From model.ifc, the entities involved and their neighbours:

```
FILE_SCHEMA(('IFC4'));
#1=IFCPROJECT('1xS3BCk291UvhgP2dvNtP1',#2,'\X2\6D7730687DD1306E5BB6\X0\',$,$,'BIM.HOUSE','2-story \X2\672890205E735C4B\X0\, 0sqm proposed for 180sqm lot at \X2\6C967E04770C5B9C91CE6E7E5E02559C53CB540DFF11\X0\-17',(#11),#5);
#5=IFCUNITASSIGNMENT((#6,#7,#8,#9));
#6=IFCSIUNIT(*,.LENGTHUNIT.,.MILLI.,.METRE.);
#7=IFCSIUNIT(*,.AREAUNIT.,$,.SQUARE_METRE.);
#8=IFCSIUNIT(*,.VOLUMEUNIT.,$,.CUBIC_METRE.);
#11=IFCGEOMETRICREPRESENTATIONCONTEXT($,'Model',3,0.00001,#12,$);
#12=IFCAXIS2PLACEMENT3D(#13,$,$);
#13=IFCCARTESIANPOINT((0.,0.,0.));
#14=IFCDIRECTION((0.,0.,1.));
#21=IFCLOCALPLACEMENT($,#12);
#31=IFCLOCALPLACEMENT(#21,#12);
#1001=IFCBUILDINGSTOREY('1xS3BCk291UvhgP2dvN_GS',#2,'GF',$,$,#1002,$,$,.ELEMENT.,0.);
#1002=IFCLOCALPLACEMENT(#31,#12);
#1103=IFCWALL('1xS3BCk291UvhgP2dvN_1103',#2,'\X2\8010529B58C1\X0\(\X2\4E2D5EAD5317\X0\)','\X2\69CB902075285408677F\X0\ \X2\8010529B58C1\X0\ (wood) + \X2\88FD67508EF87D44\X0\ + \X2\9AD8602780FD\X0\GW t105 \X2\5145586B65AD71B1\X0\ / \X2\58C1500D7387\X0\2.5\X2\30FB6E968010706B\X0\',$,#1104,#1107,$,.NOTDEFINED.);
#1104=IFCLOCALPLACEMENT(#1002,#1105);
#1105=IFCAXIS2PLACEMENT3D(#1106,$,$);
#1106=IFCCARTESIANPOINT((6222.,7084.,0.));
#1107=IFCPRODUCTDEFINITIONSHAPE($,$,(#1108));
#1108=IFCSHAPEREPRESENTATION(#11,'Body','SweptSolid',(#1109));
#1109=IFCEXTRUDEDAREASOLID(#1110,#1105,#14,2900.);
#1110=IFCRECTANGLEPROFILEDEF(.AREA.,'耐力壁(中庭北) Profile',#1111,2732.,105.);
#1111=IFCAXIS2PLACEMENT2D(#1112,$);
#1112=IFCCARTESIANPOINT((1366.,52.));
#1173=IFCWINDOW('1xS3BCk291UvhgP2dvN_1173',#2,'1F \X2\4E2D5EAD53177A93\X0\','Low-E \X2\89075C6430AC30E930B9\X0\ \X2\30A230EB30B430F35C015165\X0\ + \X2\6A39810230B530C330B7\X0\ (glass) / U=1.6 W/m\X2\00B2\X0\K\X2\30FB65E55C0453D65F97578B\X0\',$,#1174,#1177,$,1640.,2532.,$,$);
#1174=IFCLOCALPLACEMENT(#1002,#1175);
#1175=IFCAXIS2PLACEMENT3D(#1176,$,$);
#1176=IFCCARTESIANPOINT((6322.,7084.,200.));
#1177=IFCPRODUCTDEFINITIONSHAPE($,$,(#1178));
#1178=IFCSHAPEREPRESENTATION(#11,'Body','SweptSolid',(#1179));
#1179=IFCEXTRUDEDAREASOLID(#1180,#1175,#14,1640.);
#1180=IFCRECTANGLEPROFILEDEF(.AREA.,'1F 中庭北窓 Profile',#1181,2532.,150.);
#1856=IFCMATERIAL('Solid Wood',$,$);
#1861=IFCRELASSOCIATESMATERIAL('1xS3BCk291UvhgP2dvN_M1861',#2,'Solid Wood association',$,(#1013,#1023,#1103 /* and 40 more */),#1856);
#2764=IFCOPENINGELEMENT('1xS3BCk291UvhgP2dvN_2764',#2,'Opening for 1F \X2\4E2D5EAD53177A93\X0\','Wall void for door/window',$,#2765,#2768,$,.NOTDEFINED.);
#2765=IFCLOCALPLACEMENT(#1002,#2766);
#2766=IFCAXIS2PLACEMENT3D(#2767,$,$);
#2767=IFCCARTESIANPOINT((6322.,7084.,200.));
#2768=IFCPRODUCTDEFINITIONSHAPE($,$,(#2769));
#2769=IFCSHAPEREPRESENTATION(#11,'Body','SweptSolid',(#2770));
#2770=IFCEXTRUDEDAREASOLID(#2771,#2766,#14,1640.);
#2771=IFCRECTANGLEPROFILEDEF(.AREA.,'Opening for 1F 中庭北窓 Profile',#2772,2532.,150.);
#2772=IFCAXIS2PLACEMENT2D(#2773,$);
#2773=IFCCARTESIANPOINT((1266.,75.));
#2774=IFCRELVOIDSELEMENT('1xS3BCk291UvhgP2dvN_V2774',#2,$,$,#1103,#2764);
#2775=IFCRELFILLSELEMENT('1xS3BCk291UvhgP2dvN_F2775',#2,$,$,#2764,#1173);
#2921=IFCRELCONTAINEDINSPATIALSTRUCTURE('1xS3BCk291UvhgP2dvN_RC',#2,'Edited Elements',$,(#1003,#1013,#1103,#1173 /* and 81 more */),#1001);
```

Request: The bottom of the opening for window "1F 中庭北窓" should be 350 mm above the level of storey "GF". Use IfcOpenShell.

```python
import numpy as np
import ifcopenshell
import ifcopenshell.api.geometry
import ifcopenshell.geom
import ifcopenshell.util.element
import ifcopenshell.util.placement
import ifcopenshell.util.shape
import ifcopenshell.util.unit

model = ifcopenshell.open("model.ifc")
unit_scale = ifcopenshell.util.unit.calculate_unit_scale(model)

window = model.by_guid("1xS3BCk291UvhgP2dvN_1173")
opening = window.FillsVoids[0].RelatingOpeningElement
storey = ifcopenshell.util.element.get_container(window, ifc_class="IfcBuildingStorey")
level = ifcopenshell.util.placement.get_local_placement(storey.ObjectPlacement)[2, 3]

# The opening's origin need not be at the sill, so measure its lowest point.
shape = ifcopenshell.geom.create_shape(ifcopenshell.geom.settings(), opening)
bottom = ifcopenshell.util.shape.get_shape_bottom_elevation(shape, shape.geometry) / unit_scale
dz = level + 0.35 / unit_scale - bottom

shift = np.array([0.0, 0.0, dz])
# The window is not placed relative to its opening, so move both.
for product in (opening, window):
    matrix = ifcopenshell.util.placement.get_local_placement(product.ObjectPlacement)
    matrix[:3, 3] += shift
    ifcopenshell.api.geometry.edit_object_placement(model, product=product, matrix=matrix, is_si=False)

print(f"moved by {dz * unit_scale:+.3f} m")

model.write("model_edited.ifc")
```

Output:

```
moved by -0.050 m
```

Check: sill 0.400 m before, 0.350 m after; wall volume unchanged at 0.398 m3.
